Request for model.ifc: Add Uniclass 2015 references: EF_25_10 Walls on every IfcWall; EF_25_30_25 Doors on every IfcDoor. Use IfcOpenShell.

First a look at what the model holds.

```python
import ifcopenshell

model = ifcopenshell.open("model.ifc")
print(model.schema)
print("classifications:", [c.Name for c in model.by_type("IfcClassification")])
for ifc_class in ("IfcDoor", "IfcRoof", "IfcStair", "IfcWall", "IfcWindow"):
    print(ifc_class, len(model.by_type(ifc_class)))
```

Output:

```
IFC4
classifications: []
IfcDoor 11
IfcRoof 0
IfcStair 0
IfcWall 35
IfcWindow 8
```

```python
import ifcopenshell
import ifcopenshell.api.classification

model = ifcopenshell.open("model.ifc")

system = ifcopenshell.api.classification.add_classification(model, classification="Uniclass 2015")

codes = {
    "IfcWall": ("EF_25_10", "Walls"),
    "IfcDoor": ("EF_25_30_25", "Doors"),
}
for ifc_class, (code, name) in codes.items():
    products = model.by_type(ifc_class)
    ifcopenshell.api.classification.add_reference(
        model, products=products, classification=system, identification=code, name=name
    )
    print(code, len(products))

model.write("model_edited.ifc")
```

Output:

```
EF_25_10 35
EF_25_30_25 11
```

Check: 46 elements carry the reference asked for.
